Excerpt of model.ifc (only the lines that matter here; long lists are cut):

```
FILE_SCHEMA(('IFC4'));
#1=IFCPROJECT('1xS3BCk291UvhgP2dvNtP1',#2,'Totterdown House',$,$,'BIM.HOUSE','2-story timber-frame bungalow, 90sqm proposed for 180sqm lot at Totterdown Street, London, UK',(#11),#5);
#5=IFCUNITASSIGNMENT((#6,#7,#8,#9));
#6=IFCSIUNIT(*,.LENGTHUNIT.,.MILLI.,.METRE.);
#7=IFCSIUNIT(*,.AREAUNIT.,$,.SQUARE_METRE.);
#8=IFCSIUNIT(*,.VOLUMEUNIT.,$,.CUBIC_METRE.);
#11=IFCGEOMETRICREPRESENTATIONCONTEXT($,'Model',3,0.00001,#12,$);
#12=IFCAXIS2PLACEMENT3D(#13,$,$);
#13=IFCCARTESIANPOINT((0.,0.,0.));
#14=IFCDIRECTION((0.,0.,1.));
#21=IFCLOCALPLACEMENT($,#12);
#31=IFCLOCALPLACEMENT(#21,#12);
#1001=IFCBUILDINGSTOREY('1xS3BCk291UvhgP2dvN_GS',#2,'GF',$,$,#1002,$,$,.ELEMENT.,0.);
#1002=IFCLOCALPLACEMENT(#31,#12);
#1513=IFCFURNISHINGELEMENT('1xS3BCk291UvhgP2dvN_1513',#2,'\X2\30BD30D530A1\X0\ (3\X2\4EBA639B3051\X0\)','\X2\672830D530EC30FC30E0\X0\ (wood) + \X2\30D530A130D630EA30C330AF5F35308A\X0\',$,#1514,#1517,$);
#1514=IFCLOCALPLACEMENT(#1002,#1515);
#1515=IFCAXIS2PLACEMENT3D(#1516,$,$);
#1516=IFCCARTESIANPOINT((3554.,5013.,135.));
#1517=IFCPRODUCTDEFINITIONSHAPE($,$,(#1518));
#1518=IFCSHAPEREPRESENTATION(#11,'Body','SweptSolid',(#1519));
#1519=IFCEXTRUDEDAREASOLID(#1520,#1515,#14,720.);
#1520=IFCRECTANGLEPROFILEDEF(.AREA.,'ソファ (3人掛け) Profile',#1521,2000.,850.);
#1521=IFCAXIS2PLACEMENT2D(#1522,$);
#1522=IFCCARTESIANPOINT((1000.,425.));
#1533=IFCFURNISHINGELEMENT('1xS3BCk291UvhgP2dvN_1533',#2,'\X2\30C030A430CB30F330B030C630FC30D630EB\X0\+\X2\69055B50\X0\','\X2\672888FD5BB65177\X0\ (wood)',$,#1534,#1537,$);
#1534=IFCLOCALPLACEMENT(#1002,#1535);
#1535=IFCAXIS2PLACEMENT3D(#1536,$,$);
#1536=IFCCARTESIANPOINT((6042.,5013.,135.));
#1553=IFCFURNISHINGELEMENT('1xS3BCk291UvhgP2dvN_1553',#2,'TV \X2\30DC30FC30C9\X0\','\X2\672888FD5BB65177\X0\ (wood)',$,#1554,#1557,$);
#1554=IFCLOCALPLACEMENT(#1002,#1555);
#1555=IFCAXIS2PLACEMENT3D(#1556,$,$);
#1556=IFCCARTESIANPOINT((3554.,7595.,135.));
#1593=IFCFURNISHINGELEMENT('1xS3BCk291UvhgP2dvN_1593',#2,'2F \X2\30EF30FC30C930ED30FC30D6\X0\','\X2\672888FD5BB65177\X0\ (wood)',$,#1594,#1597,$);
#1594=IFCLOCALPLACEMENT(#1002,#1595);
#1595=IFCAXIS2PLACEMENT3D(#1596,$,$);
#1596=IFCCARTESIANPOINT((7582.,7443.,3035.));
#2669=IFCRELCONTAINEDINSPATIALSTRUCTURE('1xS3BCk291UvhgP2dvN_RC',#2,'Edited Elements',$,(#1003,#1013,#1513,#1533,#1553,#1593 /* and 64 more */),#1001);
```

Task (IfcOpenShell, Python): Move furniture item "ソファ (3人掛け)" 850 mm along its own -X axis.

```python
import ifcopenshell
import ifcopenshell.api.geometry
import ifcopenshell.util.placement
import ifcopenshell.util.unit

model = ifcopenshell.open("model.ifc")
unit_scale = ifcopenshell.util.unit.calculate_unit_scale(model)

item = model.by_id(1513)
matrix = ifcopenshell.util.placement.get_local_placement(item.ObjectPlacement)
matrix[:3, 3] -= matrix[:3, 0] * 0.85 / unit_scale
ifcopenshell.api.geometry.edit_object_placement(model, product=item, matrix=matrix, is_si=False)

print(ifcopenshell.util.placement.get_local_placement(item.ObjectPlacement).round(3) + 0.0)

model.write("model_v2.ifc")
```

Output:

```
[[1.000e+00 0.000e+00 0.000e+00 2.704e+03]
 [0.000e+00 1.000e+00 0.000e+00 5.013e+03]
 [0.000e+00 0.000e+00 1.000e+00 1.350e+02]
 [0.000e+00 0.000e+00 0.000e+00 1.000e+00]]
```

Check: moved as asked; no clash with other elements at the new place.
